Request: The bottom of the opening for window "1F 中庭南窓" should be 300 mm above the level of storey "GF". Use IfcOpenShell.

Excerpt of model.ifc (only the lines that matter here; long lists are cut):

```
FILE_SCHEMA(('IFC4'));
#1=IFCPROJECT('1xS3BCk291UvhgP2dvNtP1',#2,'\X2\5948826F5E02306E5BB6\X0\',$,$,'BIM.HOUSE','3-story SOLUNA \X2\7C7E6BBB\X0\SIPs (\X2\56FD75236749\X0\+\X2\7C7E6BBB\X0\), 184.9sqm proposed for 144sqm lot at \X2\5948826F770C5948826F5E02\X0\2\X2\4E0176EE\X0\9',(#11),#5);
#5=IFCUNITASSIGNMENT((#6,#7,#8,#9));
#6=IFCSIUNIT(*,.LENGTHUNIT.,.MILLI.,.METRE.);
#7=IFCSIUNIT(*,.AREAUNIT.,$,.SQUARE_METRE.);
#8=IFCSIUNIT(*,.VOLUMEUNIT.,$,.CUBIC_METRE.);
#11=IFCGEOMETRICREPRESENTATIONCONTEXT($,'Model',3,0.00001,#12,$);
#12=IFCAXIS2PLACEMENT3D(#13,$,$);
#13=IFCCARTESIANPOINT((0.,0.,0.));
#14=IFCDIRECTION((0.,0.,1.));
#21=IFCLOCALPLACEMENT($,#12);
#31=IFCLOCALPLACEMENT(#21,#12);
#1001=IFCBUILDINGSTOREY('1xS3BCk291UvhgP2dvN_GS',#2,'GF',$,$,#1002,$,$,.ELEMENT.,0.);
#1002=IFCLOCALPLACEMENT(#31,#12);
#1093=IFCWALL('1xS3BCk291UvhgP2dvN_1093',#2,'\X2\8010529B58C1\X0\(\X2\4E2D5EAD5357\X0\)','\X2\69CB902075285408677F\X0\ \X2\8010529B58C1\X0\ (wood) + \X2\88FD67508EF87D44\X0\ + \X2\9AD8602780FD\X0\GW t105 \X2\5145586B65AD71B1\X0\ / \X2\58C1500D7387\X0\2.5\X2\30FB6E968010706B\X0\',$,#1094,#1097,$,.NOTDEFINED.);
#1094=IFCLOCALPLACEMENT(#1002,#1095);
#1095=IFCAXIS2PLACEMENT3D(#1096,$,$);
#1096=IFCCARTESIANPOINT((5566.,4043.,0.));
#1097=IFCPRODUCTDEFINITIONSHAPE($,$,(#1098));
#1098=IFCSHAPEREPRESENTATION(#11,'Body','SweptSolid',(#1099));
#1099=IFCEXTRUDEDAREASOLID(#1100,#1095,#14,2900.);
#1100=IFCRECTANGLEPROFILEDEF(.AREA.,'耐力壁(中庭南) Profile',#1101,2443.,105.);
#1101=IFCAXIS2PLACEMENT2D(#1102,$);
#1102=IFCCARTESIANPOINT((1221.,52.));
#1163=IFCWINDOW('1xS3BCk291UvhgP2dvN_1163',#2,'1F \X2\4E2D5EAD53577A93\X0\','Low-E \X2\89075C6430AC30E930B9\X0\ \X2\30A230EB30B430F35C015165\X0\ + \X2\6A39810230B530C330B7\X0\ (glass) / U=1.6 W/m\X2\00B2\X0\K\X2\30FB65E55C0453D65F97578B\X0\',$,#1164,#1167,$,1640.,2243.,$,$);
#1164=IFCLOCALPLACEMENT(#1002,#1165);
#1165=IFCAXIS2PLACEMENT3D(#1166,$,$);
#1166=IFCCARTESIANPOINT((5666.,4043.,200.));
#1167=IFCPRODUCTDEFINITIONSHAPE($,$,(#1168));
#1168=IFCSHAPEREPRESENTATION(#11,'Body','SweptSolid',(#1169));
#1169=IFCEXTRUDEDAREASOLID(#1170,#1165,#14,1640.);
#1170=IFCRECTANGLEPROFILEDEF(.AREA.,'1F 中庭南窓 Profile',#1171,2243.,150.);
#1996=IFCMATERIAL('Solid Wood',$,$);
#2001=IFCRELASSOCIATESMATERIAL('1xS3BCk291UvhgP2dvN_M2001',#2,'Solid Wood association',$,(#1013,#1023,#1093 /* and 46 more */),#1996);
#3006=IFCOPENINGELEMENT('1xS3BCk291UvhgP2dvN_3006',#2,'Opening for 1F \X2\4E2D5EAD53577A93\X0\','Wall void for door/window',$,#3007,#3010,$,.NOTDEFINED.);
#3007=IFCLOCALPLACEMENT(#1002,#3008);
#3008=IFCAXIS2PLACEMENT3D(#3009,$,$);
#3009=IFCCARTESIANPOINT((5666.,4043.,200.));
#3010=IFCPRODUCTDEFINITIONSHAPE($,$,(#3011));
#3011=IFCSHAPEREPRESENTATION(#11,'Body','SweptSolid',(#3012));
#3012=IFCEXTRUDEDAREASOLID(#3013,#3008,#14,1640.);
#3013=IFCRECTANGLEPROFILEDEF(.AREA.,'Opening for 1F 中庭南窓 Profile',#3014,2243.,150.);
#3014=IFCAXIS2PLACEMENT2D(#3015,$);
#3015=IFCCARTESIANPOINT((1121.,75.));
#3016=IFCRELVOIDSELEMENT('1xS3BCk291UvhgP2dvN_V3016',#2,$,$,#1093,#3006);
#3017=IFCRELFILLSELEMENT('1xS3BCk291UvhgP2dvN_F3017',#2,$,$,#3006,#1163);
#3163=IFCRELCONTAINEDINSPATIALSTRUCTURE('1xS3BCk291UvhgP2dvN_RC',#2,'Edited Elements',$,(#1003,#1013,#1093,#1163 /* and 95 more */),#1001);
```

```python
import numpy as np
import ifcopenshell
import ifcopenshell.api.geometry
import ifcopenshell.geom
import ifcopenshell.util.element
import ifcopenshell.util.placement
import ifcopenshell.util.shape
import ifcopenshell.util.unit

model = ifcopenshell.open("model.ifc")
unit_scale = ifcopenshell.util.unit.calculate_unit_scale(model)

window = model.by_id(1163)
opening = window.FillsVoids[0].RelatingOpeningElement
storey = ifcopenshell.util.element.get_container(window, ifc_class="IfcBuildingStorey")
level = ifcopenshell.util.placement.get_local_placement(storey.ObjectPlacement)[2, 3]

# The opening's origin need not be at the sill, so measure its lowest point.
shape = ifcopenshell.geom.create_shape(ifcopenshell.geom.settings(), opening)
bottom = ifcopenshell.util.shape.get_shape_bottom_elevation(shape, shape.geometry) / unit_scale
dz = level + 300.0 - bottom

shift = np.array([0.0, 0.0, dz])
# The window is not placed relative to its opening, so move both.
for product in (opening, window):
    matrix = ifcopenshell.util.placement.get_local_placement(product.ObjectPlacement)
    matrix[:3, 3] += shift
    ifcopenshell.api.geometry.edit_object_placement(model, product=product, matrix=matrix, is_si=False)

print(f"moved by {dz * unit_scale:+.3f} m")

model.write("model_edited.ifc")
```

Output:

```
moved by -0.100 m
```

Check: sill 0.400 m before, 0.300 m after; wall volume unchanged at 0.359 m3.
